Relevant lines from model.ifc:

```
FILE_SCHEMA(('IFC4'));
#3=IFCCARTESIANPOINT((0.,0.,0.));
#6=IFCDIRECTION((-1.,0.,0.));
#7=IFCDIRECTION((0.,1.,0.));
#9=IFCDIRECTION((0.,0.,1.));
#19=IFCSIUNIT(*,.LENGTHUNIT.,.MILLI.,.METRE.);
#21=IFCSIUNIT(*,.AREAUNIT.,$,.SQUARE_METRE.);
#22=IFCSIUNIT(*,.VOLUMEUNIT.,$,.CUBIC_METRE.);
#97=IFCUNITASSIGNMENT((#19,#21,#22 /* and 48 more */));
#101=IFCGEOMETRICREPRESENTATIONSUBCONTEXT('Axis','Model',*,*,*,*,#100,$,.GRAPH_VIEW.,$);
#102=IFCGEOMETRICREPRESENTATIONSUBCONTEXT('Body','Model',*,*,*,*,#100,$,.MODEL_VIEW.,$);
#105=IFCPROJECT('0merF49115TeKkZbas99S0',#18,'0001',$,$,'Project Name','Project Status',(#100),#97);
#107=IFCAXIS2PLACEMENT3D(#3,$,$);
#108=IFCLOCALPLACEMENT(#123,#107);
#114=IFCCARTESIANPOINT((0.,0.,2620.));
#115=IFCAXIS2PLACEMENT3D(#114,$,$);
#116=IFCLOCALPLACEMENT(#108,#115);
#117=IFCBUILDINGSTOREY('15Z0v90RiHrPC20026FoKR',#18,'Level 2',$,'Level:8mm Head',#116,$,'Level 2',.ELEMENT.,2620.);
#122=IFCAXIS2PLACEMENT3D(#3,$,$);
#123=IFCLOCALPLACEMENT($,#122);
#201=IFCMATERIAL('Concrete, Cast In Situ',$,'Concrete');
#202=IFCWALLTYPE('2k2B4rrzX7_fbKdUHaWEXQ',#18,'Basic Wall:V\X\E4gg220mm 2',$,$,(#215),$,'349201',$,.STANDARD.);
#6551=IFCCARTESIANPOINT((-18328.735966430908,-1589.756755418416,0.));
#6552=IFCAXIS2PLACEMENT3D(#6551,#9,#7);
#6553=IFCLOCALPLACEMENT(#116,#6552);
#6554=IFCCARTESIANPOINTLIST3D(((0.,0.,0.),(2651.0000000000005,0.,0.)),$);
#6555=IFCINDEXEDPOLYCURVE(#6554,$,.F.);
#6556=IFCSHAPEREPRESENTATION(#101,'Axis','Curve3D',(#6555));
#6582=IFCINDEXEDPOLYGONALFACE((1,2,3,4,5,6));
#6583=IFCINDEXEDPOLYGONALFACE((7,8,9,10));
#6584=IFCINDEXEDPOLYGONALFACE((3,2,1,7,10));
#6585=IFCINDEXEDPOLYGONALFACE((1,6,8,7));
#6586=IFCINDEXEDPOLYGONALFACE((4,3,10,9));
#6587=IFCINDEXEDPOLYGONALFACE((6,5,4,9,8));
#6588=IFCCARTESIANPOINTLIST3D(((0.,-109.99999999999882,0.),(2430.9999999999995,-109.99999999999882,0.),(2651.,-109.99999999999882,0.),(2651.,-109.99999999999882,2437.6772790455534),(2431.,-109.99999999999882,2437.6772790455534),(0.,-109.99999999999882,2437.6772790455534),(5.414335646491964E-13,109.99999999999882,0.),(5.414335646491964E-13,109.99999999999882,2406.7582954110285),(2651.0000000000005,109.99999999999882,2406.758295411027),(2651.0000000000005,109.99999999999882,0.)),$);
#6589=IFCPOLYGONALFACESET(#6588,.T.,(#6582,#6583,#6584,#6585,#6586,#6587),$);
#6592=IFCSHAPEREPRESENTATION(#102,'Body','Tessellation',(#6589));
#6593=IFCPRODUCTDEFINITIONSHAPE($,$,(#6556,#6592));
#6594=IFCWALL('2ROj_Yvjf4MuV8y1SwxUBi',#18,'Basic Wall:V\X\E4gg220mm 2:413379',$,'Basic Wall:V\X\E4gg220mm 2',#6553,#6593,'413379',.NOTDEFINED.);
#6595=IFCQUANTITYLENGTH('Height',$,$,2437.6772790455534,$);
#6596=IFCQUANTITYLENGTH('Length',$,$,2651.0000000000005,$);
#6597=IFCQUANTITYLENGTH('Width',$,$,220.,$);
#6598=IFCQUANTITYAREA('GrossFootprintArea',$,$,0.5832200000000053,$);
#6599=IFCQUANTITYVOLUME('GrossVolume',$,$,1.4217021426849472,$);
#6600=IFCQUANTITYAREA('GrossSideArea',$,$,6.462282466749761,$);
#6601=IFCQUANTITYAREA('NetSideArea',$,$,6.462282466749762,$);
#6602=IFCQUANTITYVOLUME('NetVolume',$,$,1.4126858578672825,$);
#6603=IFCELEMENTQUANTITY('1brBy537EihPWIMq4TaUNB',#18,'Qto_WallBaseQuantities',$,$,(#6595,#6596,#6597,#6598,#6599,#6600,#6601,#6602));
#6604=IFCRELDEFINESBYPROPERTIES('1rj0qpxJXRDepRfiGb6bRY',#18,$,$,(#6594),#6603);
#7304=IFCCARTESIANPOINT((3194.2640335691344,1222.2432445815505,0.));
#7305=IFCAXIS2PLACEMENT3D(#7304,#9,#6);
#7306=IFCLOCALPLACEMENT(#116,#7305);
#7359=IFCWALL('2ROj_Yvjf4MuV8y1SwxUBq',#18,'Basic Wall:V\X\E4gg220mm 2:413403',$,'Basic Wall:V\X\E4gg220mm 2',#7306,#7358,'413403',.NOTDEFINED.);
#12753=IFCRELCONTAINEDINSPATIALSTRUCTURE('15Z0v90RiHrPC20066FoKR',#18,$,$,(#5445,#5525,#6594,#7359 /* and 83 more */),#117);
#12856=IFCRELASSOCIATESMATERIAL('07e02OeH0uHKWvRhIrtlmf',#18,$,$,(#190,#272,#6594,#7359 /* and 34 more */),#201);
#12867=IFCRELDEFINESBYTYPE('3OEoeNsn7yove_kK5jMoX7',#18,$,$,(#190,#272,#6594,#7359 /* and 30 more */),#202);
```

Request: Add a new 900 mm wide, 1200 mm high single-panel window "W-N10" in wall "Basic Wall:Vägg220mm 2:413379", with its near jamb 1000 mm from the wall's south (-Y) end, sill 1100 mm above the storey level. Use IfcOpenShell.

```python
import numpy as np
import ifcopenshell
import ifcopenshell.api.feature
import ifcopenshell.api.geometry
import ifcopenshell.api.pset
import ifcopenshell.api.root
import ifcopenshell.api.spatial
import ifcopenshell.geom
import ifcopenshell.util.element
import ifcopenshell.util.placement
import ifcopenshell.util.representation
import ifcopenshell.util.shape
import ifcopenshell.util.unit

model = ifcopenshell.open("model.ifc")
unit_scale = ifcopenshell.util.unit.calculate_unit_scale(model)
area_scale = ifcopenshell.util.unit.calculate_unit_scale(model, "AREAUNIT")
volume_scale = ifcopenshell.util.unit.calculate_unit_scale(model, "VOLUMEUNIT")
settings = ifcopenshell.geom.settings()


def volume(element):
    """Net volume in cubic metres, openings subtracted."""
    shape = ifcopenshell.geom.create_shape(settings, element)
    return ifcopenshell.util.shape.get_volume(shape.geometry)


wall = model.by_guid("2ROj_Yvjf4MuV8y1SwxUBi")
storey = ifcopenshell.util.element.get_container(wall, ifc_class="IfcBuildingStorey")
context = ifcopenshell.util.representation.get_context(model, "Model", "Body", "MODEL_VIEW")
before = volume(wall)

width, height, from_end, sill = 0.9, 1.2, 1, 1.1  # metres

# The wall runs along its own X axis, and the end named is its -X end.
wall_shape = ifcopenshell.geom.create_shape(settings, wall)
x, y, z = ifcopenshell.util.shape.get_vertices(wall_shape.geometry).T
start = x.min() + from_end
face, thickness = float(y.min()), float(y.max() - y.min())
wall_matrix = ifcopenshell.util.placement.get_local_placement(wall.ObjectPlacement)
level = ifcopenshell.util.placement.get_local_placement(storey.ObjectPlacement)[2, 3]


def in_wall(x, y):
    """Placement at x, y metres in the wall's axes, at sill height."""
    matrix = wall_matrix.copy()
    matrix[:, 3] = wall_matrix @ np.array([x / unit_scale, y / unit_scale, 0.0, 1.0])
    matrix[2, 3] = level + sill / unit_scale
    return matrix


# Opening: a box that overshoots both wall faces by 50 mm.
opening = ifcopenshell.api.root.create_entity(model, ifc_class="IfcOpeningElement", predefined_type="OPENING")
box = ifcopenshell.api.geometry.add_wall_representation(
    model, context=context, length=width, height=height, thickness=thickness + 0.1
)
ifcopenshell.api.geometry.assign_representation(model, product=opening, representation=box)
ifcopenshell.api.geometry.edit_object_placement(model, product=opening, matrix=in_wall(start, face - 0.05), is_si=False)
ifcopenshell.api.feature.add_feature(model, feature=opening, element=wall)

window = ifcopenshell.api.root.create_entity(model, ifc_class="IfcWindow", name="W-N10", predefined_type="WINDOW")
window.OverallWidth, window.OverallHeight = width / unit_scale, height / unit_scale
window.PartitioningType = "SINGLE_PANEL"
body = ifcopenshell.api.geometry.add_window_representation(
    model,
    context=context,
    overall_width=window.OverallWidth,
    overall_height=window.OverallHeight,
    partition_type="SINGLE_PANEL",
)
ifcopenshell.api.geometry.assign_representation(model, product=window, representation=body)
ifcopenshell.api.spatial.assign_container(model, products=[window], relating_structure=storey)
ifcopenshell.api.feature.add_filling(model, opening=opening, element=window)

# Centre the window in the wall's thickness.
ifcopenshell.api.geometry.edit_object_placement(model, product=window, matrix=in_wall(start, face), is_si=False)
window_shape = ifcopenshell.geom.create_shape(settings, window)
depth = ifcopenshell.util.shape.get_vertices(window_shape.geometry)[:, 1]
offset = face + thickness / 2 - (depth.min() + depth.max()) / 2
ifcopenshell.api.geometry.edit_object_placement(model, product=window, matrix=in_wall(start, offset), is_si=False)

after = volume(wall)

# Update the wall's stored quantities.
qto = model.by_id(ifcopenshell.util.element.get_pset(wall, "Qto_WallBaseQuantities", should_inherit=False)["id"])
ifcopenshell.api.pset.edit_qto(model, qto=qto, properties={
    "NetSideArea": after / thickness / area_scale,
    "NetVolume": after / volume_scale,
})

print(f"wall volume {before:.3f} -> {after:.3f} m3")

model.write("model_v2.ifc")
```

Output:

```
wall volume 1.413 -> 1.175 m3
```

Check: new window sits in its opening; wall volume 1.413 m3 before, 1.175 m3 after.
